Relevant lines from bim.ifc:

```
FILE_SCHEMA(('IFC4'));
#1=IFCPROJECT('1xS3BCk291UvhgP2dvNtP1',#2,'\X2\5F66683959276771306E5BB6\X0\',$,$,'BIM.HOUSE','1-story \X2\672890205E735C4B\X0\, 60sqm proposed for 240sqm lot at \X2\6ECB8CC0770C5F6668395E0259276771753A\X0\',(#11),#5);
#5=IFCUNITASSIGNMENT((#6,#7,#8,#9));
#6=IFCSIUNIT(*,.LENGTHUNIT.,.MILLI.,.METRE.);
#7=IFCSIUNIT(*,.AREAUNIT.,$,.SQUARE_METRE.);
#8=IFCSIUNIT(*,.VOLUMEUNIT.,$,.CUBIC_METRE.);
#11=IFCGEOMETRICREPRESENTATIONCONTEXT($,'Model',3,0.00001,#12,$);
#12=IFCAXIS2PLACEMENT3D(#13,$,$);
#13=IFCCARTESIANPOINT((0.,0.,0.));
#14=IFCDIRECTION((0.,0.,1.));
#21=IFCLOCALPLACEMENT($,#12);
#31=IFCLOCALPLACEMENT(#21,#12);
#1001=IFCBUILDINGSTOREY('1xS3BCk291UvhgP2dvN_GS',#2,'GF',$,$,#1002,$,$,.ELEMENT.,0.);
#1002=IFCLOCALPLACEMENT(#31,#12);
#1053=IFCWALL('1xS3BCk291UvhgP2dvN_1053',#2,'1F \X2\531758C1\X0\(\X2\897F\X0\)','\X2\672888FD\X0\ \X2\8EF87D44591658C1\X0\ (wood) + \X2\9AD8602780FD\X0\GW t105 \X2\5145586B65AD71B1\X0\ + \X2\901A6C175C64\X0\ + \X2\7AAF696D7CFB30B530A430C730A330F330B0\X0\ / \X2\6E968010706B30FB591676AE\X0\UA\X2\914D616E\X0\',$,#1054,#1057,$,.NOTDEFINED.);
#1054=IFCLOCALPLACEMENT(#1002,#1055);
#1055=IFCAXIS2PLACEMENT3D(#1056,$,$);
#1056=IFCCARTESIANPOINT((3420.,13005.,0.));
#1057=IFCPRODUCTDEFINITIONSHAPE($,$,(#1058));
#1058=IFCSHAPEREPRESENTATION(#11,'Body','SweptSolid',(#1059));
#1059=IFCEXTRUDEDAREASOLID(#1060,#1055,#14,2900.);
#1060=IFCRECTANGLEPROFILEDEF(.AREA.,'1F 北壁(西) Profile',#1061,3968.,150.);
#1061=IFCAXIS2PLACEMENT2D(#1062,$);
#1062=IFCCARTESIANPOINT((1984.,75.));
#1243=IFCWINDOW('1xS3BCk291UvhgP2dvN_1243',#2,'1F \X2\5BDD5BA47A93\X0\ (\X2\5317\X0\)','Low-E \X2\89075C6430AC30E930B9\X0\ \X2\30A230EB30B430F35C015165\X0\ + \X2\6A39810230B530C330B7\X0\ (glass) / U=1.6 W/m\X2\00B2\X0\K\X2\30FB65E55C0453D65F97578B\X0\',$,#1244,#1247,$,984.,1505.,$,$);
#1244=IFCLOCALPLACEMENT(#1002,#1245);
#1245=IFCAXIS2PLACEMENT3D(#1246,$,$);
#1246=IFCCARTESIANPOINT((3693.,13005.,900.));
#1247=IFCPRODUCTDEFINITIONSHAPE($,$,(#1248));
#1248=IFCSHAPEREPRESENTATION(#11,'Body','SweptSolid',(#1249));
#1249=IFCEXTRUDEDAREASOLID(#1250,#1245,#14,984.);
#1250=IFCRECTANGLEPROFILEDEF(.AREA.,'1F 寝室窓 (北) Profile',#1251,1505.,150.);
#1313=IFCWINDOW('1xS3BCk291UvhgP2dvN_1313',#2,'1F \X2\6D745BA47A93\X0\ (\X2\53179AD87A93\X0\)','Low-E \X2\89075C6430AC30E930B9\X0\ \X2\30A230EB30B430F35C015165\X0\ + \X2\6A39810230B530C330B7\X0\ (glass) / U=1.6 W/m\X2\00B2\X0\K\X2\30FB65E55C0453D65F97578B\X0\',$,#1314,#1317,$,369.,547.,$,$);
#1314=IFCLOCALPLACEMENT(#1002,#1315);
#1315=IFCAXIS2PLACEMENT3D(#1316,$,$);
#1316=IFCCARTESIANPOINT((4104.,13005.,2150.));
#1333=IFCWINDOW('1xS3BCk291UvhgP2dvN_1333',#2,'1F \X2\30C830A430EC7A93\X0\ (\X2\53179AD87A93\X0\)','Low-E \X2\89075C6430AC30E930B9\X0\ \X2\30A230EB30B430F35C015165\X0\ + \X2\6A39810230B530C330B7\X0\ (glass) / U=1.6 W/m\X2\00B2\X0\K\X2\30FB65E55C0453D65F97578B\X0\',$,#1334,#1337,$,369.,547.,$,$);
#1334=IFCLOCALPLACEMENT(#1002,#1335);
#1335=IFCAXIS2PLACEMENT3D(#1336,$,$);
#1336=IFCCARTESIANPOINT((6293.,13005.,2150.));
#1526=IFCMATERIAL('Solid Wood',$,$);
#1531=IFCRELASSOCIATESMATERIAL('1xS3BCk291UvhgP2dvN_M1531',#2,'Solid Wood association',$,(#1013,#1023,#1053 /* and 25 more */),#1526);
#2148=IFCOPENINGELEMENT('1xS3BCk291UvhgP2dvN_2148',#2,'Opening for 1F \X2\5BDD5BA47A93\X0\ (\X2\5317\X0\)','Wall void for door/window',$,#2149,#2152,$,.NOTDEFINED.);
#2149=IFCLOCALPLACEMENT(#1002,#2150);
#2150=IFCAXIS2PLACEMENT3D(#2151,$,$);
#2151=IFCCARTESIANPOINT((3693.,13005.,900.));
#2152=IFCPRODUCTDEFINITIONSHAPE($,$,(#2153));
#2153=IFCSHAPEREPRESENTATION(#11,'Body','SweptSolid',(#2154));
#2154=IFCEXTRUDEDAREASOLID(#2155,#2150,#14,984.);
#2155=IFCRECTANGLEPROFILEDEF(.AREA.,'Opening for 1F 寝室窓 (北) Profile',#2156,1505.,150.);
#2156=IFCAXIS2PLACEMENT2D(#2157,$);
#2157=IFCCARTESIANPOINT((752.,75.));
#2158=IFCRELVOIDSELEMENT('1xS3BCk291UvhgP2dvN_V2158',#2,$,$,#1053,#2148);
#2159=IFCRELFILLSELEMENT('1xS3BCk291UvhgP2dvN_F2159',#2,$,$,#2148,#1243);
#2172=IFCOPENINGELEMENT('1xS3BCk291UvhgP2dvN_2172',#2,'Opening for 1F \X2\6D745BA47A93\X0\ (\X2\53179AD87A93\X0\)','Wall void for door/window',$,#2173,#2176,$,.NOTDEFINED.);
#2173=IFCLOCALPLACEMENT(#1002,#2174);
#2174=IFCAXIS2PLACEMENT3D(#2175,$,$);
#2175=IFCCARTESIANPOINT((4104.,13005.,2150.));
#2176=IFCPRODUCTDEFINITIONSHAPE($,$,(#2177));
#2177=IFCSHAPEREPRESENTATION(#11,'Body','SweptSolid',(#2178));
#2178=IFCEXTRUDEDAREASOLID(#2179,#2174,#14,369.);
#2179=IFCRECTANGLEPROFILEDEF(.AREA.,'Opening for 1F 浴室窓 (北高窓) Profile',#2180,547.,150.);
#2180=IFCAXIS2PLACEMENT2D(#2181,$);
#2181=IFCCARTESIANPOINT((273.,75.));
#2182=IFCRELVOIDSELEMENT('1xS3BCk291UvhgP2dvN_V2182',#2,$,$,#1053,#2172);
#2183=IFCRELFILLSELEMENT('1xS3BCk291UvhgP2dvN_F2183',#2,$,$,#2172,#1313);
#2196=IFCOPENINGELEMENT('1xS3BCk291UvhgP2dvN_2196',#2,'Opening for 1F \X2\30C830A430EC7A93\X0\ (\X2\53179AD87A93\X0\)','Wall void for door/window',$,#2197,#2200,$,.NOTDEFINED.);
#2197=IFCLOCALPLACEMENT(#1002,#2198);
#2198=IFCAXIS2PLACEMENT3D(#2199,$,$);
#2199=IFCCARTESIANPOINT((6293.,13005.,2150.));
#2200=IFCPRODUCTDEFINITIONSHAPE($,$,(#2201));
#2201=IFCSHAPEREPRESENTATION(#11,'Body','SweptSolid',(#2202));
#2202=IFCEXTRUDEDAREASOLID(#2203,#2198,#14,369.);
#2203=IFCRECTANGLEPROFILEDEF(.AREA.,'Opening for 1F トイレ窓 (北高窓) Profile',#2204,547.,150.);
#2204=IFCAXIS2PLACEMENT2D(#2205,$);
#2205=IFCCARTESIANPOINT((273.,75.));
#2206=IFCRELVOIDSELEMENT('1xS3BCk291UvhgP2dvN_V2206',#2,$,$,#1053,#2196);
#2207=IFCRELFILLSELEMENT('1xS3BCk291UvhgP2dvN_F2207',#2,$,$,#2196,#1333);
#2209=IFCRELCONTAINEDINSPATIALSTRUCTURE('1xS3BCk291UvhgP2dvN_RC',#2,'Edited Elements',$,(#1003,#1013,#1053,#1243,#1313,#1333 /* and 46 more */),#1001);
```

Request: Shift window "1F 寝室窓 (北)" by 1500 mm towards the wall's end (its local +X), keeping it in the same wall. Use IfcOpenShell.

```python
import ifcopenshell
import ifcopenshell.api.geometry
import ifcopenshell.util.placement
import ifcopenshell.util.unit

model = ifcopenshell.open("bim.ifc")
unit_scale = ifcopenshell.util.unit.calculate_unit_scale(model)

window = model.by_id(1243)
opening = window.FillsVoids[0].RelatingOpeningElement
wall = opening.VoidsElements[0].RelatingBuildingElement

wall_matrix = ifcopenshell.util.placement.get_local_placement(wall.ObjectPlacement)
shift = wall_matrix[:3, 0] * 1.5 / unit_scale
before = ifcopenshell.util.placement.get_local_placement(window.ObjectPlacement)[:3, 3].copy()

# The window is not placed relative to its opening, so move both.
for product in (opening, window):
    matrix = ifcopenshell.util.placement.get_local_placement(product.ObjectPlacement)
    matrix[:3, 3] += shift
    ifcopenshell.api.geometry.edit_object_placement(model, product=product, matrix=matrix, is_si=False)

after = ifcopenshell.util.placement.get_local_placement(window.ObjectPlacement)[:3, 3]
print("window moved by", (after - before).round(3) + 0.0)

model.write("bim_rev.ifc")
```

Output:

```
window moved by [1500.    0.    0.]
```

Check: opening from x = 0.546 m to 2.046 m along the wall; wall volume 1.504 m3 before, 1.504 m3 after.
